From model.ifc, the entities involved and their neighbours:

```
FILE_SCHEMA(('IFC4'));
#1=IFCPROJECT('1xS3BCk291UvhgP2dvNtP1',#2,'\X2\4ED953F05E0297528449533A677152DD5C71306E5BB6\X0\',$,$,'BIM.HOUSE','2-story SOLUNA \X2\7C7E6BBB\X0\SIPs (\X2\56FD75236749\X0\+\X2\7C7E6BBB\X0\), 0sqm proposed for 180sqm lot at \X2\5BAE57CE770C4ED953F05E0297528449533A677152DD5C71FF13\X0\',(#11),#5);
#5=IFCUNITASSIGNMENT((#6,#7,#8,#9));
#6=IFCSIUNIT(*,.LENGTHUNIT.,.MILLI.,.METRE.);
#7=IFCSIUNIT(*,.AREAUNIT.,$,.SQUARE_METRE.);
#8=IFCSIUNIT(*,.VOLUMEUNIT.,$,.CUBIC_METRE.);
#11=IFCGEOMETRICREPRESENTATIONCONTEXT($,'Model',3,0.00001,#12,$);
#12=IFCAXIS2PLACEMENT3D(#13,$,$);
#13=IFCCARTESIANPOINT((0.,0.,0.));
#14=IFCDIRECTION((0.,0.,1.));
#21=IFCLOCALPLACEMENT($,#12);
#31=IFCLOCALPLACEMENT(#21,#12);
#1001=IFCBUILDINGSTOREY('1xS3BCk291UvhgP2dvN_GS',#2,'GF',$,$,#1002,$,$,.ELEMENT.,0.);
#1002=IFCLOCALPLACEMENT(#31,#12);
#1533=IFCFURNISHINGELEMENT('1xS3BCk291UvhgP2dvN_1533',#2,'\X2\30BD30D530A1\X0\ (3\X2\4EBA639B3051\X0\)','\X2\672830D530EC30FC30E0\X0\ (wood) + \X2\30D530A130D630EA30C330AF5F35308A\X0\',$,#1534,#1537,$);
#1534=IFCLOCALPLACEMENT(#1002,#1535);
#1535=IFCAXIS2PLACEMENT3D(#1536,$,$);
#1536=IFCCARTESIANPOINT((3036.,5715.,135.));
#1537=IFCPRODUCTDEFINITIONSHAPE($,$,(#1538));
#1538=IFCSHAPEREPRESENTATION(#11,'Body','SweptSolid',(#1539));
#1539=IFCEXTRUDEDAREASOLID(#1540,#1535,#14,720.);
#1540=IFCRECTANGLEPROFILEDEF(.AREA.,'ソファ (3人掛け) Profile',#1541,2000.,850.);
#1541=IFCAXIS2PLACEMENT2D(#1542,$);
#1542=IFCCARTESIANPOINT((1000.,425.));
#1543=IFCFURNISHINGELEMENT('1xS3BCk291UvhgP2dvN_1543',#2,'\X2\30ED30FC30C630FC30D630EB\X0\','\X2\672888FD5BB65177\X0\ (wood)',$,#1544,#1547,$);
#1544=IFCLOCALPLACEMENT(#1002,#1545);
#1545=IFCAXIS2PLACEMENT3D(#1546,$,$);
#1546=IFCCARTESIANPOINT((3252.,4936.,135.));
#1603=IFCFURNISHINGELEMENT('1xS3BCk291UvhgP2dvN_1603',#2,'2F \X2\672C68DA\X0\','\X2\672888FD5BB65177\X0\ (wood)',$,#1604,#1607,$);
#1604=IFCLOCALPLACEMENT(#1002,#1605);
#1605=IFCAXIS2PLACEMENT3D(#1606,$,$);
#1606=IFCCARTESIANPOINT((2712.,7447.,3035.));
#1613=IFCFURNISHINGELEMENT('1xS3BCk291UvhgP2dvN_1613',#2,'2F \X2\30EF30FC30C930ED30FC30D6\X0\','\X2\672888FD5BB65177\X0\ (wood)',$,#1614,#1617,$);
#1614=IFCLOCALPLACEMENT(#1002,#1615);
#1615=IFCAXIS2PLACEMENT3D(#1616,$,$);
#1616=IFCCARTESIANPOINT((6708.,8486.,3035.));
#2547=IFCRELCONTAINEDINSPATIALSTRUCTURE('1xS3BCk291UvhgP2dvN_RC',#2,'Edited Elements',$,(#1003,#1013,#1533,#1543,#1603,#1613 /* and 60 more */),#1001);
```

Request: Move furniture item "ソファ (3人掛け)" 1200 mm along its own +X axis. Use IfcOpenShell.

```python
import ifcopenshell
import ifcopenshell.api.geometry
import ifcopenshell.util.placement
import ifcopenshell.util.unit

model = ifcopenshell.open("model.ifc")
unit_scale = ifcopenshell.util.unit.calculate_unit_scale(model)

item = model.by_guid("1xS3BCk291UvhgP2dvN_1533")
matrix = ifcopenshell.util.placement.get_local_placement(item.ObjectPlacement)
matrix[:3, 3] += matrix[:3, 0] * 1.2 / unit_scale
ifcopenshell.api.geometry.edit_object_placement(model, product=item, matrix=matrix, is_si=False)

print(ifcopenshell.util.placement.get_local_placement(item.ObjectPlacement).round(3) + 0.0)

model.write("model_v2.ifc")
```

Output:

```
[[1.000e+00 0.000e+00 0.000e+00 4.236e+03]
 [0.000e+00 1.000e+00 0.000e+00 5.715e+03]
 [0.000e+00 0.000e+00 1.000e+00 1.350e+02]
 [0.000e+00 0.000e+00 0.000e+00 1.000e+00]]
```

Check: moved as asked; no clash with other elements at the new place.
